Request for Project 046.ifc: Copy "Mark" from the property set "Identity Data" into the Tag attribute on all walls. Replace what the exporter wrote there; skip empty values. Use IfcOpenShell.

First a look at what the model holds.

```python
import ifcopenshell
import ifcopenshell.util.element

model = ifcopenshell.open("Project 046.ifc")
print(model.schema)
walls = model.by_type("IfcWall")
print(len(walls), "walls")
for e in walls[:8]:
    source = ifcopenshell.util.element.get_pset(e, "Identity Data", "Mark")
    target = e.Tag
    print(e.id(), repr(source), repr(target), sep=" | ")
```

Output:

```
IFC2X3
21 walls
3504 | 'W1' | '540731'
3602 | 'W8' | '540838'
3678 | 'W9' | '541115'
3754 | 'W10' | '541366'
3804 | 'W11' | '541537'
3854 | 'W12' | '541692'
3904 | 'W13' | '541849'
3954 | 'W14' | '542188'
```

```python
import ifcopenshell
import ifcopenshell.util.element

model = ifcopenshell.open("Project 046.ifc")

count = 0
for e in model.by_type("IfcWall"):
    value = ifcopenshell.util.element.get_pset(e, "Identity Data", "Mark")
    current = e.Tag
    if not value or not value.strip() or current == value:
        continue
    e.Tag = value
    count += 1

print(count, "walls updated")

model.write("Project 046_rev.ifc")
```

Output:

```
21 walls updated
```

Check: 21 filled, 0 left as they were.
